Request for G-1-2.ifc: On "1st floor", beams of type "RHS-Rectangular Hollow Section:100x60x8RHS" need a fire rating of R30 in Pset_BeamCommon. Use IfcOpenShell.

First a look at what the model holds.

```python
import ifcopenshell
import ifcopenshell.util.element

model = ifcopenshell.open("G-1-2.ifc")
print(model.schema)
storey = next(s for s in model.by_type("IfcBuildingStorey") if s.Name == "1st floor")
beams = [e for e in ifcopenshell.util.element.get_decomposition(storey) if e.is_a("IfcBeam")]
seen = {}
for e in beams:
    element_type = ifcopenshell.util.element.get_type(e)
    key = (element_type.Name if element_type != e and element_type else None, ifcopenshell.util.element.get_pset(e, "Pset_BeamCommon", "FireRating"))
    seen[key] = seen.get(key, 0) + 1
for (name, value), count in sorted(seen.items(), key=str):
    print(count, "x", name, "|", value)
```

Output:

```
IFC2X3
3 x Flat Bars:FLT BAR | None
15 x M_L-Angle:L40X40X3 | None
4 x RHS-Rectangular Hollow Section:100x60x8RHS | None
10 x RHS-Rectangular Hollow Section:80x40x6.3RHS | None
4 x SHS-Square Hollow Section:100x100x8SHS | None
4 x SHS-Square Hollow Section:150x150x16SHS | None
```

```python
import ifcopenshell
import ifcopenshell.api.pset
import ifcopenshell.util.element

model = ifcopenshell.open("G-1-2.ifc")

storey = next(s for s in model.by_type("IfcBuildingStorey") if s.Name == "1st floor")
beams = [e for e in ifcopenshell.util.element.get_decomposition(storey) if e.is_a("IfcBeam")]

count = 0
for e in beams:
    element_type = ifcopenshell.util.element.get_type(e)
    if element_type in (None, e) or element_type.Name != "RHS-Rectangular Hollow Section:100x60x8RHS":
        continue
    # add_pset returns the element's existing set when there is one.
    pset = ifcopenshell.api.pset.add_pset(model, product=e, name="Pset_BeamCommon")
    ifcopenshell.api.pset.edit_pset(model, pset=pset, properties={"FireRating": "R30"})
    count += 1

print(count, "beams updated")

model.write("G-1-2_edited.ifc")
```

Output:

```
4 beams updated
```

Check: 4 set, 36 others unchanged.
